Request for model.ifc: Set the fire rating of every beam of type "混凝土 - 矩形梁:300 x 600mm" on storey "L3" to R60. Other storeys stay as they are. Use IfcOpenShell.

First a look at what the model holds.

```python
import ifcopenshell
import ifcopenshell.util.element

model = ifcopenshell.open("model.ifc")
print(model.schema)
storey = next(s for s in model.by_type("IfcBuildingStorey") if s.Name == "L3")
beams = [e for e in ifcopenshell.util.element.get_decomposition(storey) if e.is_a("IfcBeam")]
seen = {}
for e in beams:
    element_type = ifcopenshell.util.element.get_type(e)
    key = (element_type.Name if element_type != e and element_type else None, ifcopenshell.util.element.get_pset(e, "Pset_BeamCommon", "FireRating"))
    seen[key] = seen.get(key, 0) + 1
for (name, value), count in sorted(seen.items(), key=str):
    print(count, "x", name, "|", value)
```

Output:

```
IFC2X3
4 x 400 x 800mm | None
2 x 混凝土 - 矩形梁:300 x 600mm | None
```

```python
import ifcopenshell
import ifcopenshell.api.pset
import ifcopenshell.util.element

model = ifcopenshell.open("model.ifc")

storey = next(s for s in model.by_type("IfcBuildingStorey") if s.Name == "L3")
beams = [e for e in ifcopenshell.util.element.get_decomposition(storey) if e.is_a("IfcBeam")]

count = 0
for e in beams:
    element_type = ifcopenshell.util.element.get_type(e)
    if element_type in (None, e) or element_type.Name != "混凝土 - 矩形梁:300 x 600mm":
        continue
    # add_pset returns the element's existing set when there is one.
    pset = ifcopenshell.api.pset.add_pset(model, product=e, name="Pset_BeamCommon")
    ifcopenshell.api.pset.edit_pset(model, pset=pset, properties={"FireRating": "R60"})
    count += 1

print(count, "beams updated")

model.write("model_updated.ifc")
```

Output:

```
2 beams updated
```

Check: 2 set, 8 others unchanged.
